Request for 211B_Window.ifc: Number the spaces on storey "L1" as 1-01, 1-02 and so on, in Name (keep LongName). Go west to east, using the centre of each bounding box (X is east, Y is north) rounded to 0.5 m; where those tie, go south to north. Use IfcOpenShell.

First a look at what the model holds.

```python
import ifcopenshell
import ifcopenshell.util.element
import ifcopenshell.util.placement

model = ifcopenshell.open("211B_Window.ifc")
print(model.schema)
storey = next(s for s in model.by_type("IfcBuildingStorey") if s.Name == "L1")
spaces = [e for e in ifcopenshell.util.element.get_decomposition(storey) if e.is_a("IfcSpace")]
for e in sorted(spaces, key=lambda e: e.id()):
    origin = ifcopenshell.util.placement.get_local_placement(e.ObjectPlacement)[:3, 3]
    print(e.id(), e.Name, e.LongName, origin.round(2) + 0.0, sep=" | ")
```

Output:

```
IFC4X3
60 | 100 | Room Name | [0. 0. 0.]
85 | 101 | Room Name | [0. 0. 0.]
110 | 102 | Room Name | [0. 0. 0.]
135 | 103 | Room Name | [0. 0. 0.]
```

```python
import ifcopenshell
import ifcopenshell.geom
import ifcopenshell.util.element
import ifcopenshell.util.shape

model = ifcopenshell.open("211B_Window.ifc")
settings = ifcopenshell.geom.settings()
settings.set("use-world-coords", True)


def centre(element):
    shape = ifcopenshell.geom.create_shape(settings, element)
    return ifcopenshell.util.shape.get_bbox_centroid(shape.geometry)


storey = next(s for s in model.by_type("IfcBuildingStorey") if s.Name == "L1")
spaces = [e for e in ifcopenshell.util.element.get_decomposition(storey) if e.is_a("IfcSpace")]

# Insertion points can sit at a corner or the storey origin, so sort by the geometry (in metres).
centres = {e: centre(e) for e in spaces}
spaces.sort(key=lambda e: (round(centres[e][0] / 0.5), centres[e][1]))

for i, e in enumerate(spaces, start=1):
    number = f"1-{i:02d}"
    e.Name = number
    print(e.id(), number)

model.write("211B_Window_rev.ifc")
```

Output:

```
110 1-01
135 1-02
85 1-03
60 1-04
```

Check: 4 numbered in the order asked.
